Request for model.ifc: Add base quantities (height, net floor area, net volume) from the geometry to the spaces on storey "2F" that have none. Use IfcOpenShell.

First a look at what the model holds.

```python
import ifcopenshell
import ifcopenshell.util.element
import ifcopenshell.util.unit

model = ifcopenshell.open("model.ifc")
print(model.schema)
for unit_type in ("LENGTHUNIT", "AREAUNIT", "VOLUMEUNIT"):
    print(unit_type, ifcopenshell.util.unit.calculate_unit_scale(model, unit_type))
storey = next(s for s in model.by_type("IfcBuildingStorey") if s.Name == "2F")
spaces = [e for e in ifcopenshell.util.element.get_decomposition(storey) if e.is_a("IfcSpace")]
for e in sorted(spaces, key=lambda e: e.id()):
    print(e.id(), e.is_a(), e.Name, list(ifcopenshell.util.element.get_psets(e, qtos_only=True)), sep=" | ")
```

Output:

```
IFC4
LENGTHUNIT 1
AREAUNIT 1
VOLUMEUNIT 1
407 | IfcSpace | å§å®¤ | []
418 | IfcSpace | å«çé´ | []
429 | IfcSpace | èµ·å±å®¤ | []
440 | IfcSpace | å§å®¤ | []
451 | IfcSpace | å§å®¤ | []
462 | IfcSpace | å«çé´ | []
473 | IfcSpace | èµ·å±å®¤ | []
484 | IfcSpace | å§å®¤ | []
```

```python
import ifcopenshell
import ifcopenshell.api.pset
import ifcopenshell.geom
import ifcopenshell.util.element
import ifcopenshell.util.shape
import ifcopenshell.util.unit

model = ifcopenshell.open("model.ifc")
unit_scale = ifcopenshell.util.unit.calculate_unit_scale(model)
area_scale = ifcopenshell.util.unit.calculate_unit_scale(model, "AREAUNIT")
volume_scale = ifcopenshell.util.unit.calculate_unit_scale(model, "VOLUMEUNIT")
settings = ifcopenshell.geom.settings()

storey = next(s for s in model.by_type("IfcBuildingStorey") if s.Name == "2F")
spaces = [e for e in ifcopenshell.util.element.get_decomposition(storey) if e.is_a("IfcSpace")]

for e in sorted(spaces, key=lambda e: e.id()):
    if ifcopenshell.util.element.get_psets(e, qtos_only=True, should_inherit=False):
        continue
    # Geometry comes back in metres, in the element's own axes.
    shape = ifcopenshell.geom.create_shape(settings, e)
    values = {
        "Height": ifcopenshell.util.shape.get_z(shape.geometry) / unit_scale,
        "NetFloorArea": ifcopenshell.util.shape.get_footprint_area(shape.geometry) / area_scale,
        "NetVolume": ifcopenshell.util.shape.get_volume(shape.geometry) / volume_scale,
    }
    qto = ifcopenshell.api.pset.add_qto(model, product=e, name="Qto_SpaceBaseQuantities")
    ifcopenshell.api.pset.edit_qto(model, qto=qto, properties=values)
    print(e.id(), {k: round(v, 3) for k, v in values.items()})

model.write("model-out.ifc")
```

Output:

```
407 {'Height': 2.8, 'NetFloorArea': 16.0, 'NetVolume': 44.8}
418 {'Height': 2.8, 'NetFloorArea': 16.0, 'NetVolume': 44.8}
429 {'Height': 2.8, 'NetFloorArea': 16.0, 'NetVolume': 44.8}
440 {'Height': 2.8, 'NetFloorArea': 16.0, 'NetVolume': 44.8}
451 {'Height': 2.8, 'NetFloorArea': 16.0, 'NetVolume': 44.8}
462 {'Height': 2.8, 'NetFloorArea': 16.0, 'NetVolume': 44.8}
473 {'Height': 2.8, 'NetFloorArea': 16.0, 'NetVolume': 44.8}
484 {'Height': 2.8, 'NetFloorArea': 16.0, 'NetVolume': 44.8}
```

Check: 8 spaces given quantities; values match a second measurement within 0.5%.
